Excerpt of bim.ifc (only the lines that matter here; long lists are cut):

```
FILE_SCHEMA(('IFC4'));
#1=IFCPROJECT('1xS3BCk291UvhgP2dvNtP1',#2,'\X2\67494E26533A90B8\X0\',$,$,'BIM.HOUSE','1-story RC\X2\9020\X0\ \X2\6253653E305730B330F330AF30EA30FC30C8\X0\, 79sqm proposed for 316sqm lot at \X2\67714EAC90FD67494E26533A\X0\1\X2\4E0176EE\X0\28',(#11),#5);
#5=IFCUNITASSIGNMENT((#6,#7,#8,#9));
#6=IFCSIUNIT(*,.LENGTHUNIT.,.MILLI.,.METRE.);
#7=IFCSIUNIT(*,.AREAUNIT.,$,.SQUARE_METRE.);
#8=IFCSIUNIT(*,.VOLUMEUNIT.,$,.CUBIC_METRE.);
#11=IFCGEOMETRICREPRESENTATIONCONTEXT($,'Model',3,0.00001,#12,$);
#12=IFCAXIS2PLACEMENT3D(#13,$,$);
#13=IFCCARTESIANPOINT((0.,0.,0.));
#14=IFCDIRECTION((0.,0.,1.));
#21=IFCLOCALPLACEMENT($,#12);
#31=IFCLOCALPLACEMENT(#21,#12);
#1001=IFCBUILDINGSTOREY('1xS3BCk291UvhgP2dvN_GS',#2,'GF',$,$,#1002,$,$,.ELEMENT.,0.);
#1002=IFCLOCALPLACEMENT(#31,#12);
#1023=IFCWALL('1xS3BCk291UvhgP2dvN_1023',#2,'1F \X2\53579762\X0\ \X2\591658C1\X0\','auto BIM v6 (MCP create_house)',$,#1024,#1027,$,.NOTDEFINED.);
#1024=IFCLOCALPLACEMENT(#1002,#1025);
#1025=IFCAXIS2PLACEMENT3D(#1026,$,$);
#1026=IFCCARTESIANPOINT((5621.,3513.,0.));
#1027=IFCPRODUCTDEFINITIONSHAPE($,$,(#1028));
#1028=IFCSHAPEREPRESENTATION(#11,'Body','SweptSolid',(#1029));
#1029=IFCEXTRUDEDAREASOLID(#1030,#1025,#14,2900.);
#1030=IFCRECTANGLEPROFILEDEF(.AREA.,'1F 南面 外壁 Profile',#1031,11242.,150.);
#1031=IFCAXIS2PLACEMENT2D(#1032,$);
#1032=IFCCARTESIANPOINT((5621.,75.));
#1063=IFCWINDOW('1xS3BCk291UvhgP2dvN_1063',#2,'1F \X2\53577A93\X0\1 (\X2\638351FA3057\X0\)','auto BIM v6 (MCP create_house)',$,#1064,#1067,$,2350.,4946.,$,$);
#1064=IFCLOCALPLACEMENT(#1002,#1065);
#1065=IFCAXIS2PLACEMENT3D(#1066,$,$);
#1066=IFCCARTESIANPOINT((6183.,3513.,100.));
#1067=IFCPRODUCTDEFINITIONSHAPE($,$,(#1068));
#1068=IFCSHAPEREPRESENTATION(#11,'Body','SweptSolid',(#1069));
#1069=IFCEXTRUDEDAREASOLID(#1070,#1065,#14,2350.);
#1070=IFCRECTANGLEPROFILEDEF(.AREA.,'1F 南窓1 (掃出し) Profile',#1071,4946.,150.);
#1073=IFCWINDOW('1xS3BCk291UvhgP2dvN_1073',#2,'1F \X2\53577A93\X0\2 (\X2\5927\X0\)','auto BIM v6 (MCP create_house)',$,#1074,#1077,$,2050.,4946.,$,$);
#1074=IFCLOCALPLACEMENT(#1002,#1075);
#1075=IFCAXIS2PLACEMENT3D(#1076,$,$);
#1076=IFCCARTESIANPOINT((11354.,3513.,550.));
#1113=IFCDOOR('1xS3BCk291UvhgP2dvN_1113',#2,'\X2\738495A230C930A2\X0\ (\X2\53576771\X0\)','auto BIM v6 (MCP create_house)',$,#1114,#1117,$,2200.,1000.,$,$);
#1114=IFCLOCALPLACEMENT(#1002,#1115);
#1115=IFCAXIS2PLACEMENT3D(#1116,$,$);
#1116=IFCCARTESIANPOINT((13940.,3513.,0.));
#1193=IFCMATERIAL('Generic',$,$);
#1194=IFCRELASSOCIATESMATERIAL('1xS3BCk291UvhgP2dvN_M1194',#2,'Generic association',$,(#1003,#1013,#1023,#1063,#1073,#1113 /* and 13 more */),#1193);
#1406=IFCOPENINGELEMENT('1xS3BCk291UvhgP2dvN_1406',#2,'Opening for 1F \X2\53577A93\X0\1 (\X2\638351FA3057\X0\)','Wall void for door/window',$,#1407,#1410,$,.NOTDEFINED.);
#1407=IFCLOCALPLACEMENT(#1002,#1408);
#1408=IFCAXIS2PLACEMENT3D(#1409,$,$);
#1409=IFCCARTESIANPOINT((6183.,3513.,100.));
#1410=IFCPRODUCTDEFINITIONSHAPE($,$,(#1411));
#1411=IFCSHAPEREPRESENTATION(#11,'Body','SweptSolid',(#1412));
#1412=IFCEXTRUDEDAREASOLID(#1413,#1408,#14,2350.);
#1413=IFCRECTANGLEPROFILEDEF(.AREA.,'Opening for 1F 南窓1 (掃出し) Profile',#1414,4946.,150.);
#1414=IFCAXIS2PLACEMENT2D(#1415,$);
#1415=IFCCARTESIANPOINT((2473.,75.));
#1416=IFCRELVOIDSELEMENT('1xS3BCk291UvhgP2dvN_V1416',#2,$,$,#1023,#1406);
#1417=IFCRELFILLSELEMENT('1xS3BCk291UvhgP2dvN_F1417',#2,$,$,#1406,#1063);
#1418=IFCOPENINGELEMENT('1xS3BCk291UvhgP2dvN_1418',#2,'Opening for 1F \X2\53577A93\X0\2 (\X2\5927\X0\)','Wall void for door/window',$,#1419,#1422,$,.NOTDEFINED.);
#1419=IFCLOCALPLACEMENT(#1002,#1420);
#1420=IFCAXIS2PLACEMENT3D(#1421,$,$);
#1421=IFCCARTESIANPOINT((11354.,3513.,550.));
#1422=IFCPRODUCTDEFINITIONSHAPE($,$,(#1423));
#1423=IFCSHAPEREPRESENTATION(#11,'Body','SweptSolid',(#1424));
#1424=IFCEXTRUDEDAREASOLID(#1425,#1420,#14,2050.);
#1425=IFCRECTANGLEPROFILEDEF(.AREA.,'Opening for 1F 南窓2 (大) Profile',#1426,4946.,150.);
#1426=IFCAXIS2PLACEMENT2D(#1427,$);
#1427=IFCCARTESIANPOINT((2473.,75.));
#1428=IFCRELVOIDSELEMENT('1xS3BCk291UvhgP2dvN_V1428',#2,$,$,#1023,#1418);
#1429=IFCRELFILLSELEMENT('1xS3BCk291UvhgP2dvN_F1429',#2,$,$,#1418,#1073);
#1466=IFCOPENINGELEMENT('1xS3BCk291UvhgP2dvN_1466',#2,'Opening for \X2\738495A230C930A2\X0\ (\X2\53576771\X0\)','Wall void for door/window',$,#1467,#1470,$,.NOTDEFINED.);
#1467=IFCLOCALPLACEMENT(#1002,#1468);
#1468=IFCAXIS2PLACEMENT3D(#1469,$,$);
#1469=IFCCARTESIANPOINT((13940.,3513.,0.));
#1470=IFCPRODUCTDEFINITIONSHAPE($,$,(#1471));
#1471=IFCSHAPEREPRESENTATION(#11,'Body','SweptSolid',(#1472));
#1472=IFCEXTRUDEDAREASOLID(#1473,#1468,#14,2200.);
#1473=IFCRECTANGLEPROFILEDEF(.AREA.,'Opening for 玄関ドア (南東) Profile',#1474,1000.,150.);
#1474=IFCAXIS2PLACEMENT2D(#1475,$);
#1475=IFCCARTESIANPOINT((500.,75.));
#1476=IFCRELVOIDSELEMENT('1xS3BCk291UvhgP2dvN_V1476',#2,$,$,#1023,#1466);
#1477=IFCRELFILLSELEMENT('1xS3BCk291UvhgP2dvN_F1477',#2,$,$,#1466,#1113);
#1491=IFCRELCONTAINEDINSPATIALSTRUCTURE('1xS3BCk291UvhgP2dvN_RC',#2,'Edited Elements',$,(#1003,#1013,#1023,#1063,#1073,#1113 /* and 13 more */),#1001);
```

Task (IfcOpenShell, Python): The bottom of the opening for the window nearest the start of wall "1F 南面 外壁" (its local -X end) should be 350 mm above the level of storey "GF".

```python
import numpy as np
import ifcopenshell
import ifcopenshell.api.geometry
import ifcopenshell.geom
import ifcopenshell.util.element
import ifcopenshell.util.placement
import ifcopenshell.util.shape
import ifcopenshell.util.unit

model = ifcopenshell.open("bim.ifc")
unit_scale = ifcopenshell.util.unit.calculate_unit_scale(model)

window = model.by_id(1063)
opening = window.FillsVoids[0].RelatingOpeningElement
storey = ifcopenshell.util.element.get_container(window, ifc_class="IfcBuildingStorey")
level = ifcopenshell.util.placement.get_local_placement(storey.ObjectPlacement)[2, 3]

# The opening's origin need not be at the sill, so measure its lowest point.
shape = ifcopenshell.geom.create_shape(ifcopenshell.geom.settings(), opening)
bottom = ifcopenshell.util.shape.get_shape_bottom_elevation(shape, shape.geometry) / unit_scale
dz = level + 350.0 - bottom

shift = np.array([0.0, 0.0, dz])
# The window is not placed relative to its opening, so move both.
for product in (opening, window):
    matrix = ifcopenshell.util.placement.get_local_placement(product.ObjectPlacement)
    matrix[:3, 3] += shift
    ifcopenshell.api.geometry.edit_object_placement(model, product=product, matrix=matrix, is_si=False)

print(f"moved by {dz * unit_scale:+.3f} m")

model.write("bim_rev.ifc")
```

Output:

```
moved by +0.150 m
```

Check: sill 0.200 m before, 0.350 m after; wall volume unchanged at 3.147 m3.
